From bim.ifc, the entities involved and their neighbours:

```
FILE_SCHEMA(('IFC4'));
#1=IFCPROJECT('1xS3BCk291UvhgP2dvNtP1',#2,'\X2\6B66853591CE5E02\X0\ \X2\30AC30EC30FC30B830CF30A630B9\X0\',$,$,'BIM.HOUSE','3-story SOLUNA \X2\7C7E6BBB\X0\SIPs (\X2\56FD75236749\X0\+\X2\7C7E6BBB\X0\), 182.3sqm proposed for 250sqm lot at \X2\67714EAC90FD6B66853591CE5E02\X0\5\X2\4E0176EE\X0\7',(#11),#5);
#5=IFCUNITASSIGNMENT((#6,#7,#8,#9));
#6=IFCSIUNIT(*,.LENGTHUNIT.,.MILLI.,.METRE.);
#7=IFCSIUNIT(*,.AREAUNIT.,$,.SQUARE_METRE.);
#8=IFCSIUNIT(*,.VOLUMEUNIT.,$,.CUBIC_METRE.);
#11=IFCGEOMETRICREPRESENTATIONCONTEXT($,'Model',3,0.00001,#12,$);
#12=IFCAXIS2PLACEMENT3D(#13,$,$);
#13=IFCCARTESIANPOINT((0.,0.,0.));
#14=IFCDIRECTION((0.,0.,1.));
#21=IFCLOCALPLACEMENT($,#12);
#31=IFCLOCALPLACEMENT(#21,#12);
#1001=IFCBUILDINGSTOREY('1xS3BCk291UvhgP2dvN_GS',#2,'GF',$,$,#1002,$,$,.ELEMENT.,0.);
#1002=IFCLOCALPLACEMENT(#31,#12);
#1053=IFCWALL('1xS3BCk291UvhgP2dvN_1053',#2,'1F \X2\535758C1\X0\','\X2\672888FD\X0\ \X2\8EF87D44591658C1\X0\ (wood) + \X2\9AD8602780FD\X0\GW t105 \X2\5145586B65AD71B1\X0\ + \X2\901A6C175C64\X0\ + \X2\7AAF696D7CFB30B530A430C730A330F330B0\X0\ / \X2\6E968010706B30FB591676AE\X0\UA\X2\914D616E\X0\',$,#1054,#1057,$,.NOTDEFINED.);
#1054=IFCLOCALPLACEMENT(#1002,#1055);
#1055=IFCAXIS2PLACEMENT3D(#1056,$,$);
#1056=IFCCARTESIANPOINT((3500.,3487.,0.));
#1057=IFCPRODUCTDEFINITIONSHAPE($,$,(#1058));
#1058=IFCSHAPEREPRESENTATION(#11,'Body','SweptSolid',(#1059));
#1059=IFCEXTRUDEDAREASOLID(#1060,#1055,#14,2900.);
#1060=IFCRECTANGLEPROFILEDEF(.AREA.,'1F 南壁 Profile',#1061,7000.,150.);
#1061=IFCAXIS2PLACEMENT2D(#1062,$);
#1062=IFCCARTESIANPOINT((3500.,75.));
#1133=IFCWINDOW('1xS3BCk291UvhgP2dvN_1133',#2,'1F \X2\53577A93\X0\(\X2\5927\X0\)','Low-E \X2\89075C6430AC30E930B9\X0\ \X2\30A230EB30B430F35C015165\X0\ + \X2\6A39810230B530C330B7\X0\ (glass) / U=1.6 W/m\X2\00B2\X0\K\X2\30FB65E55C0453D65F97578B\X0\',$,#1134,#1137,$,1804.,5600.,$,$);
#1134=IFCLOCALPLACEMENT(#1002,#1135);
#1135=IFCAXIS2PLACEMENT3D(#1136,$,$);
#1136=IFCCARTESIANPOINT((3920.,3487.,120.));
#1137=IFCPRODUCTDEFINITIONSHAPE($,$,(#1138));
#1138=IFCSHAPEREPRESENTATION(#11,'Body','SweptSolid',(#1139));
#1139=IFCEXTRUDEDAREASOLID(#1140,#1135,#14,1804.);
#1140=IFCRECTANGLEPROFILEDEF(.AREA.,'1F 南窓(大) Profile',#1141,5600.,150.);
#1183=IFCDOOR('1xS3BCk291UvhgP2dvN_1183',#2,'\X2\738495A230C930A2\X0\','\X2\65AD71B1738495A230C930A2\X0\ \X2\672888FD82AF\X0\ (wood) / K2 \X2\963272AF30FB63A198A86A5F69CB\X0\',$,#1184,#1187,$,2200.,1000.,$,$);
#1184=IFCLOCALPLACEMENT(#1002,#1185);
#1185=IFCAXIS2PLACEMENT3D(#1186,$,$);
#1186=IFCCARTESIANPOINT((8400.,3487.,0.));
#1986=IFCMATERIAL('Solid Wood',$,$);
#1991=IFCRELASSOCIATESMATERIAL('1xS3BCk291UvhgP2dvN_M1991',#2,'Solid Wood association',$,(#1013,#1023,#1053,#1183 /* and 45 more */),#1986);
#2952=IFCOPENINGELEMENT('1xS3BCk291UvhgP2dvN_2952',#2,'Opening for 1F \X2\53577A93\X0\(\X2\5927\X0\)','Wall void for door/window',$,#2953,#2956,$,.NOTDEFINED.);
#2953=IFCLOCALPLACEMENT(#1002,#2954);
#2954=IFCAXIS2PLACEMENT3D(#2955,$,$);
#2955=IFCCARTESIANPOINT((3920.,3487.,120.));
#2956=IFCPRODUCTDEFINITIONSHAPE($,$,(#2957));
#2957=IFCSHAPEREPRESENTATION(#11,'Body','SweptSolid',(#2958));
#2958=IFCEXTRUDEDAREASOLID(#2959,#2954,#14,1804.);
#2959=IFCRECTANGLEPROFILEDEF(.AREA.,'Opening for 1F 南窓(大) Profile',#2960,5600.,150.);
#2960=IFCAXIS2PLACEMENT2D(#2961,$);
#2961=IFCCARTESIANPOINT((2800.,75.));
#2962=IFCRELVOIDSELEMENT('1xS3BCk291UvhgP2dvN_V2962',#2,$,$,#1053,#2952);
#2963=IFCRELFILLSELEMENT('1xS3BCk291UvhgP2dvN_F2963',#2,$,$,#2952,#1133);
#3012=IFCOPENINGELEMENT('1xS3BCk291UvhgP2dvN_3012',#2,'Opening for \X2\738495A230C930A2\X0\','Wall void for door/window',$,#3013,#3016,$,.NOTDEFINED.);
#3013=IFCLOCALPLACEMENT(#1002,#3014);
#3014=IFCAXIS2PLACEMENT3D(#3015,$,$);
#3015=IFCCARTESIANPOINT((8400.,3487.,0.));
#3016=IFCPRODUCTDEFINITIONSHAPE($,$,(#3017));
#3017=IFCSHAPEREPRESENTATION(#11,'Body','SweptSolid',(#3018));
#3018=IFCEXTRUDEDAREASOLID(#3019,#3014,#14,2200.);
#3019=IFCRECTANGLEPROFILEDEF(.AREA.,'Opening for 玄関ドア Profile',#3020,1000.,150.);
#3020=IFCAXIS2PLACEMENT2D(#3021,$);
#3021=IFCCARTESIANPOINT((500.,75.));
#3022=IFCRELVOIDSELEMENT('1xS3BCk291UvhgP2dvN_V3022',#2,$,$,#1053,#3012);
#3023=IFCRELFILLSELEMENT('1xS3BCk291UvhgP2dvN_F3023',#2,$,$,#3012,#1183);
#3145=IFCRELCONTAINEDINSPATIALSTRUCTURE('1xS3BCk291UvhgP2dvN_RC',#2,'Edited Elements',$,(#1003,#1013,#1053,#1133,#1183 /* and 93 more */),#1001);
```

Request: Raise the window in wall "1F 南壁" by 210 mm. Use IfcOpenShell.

```python
import numpy as np
import ifcopenshell
import ifcopenshell.api.geometry
import ifcopenshell.util.placement
import ifcopenshell.util.unit

model = ifcopenshell.open("bim.ifc")
unit_scale = ifcopenshell.util.unit.calculate_unit_scale(model)

window = model.by_guid("1xS3BCk291UvhgP2dvN_1133")
opening = window.FillsVoids[0].RelatingOpeningElement
dz = 210.0

shift = np.array([0.0, 0.0, dz])
# The window is not placed relative to its opening, so move both.
for product in (opening, window):
    matrix = ifcopenshell.util.placement.get_local_placement(product.ObjectPlacement)
    matrix[:3, 3] += shift
    ifcopenshell.api.geometry.edit_object_placement(model, product=product, matrix=matrix, is_si=False)

print(f"moved by {dz * unit_scale:+.3f} m")

model.write("bim_updated.ifc")
```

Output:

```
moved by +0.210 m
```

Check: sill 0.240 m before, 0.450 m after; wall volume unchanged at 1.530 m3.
